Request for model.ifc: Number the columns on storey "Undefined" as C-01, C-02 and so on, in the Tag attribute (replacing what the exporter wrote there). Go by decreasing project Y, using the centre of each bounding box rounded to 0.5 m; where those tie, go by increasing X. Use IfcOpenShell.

First a look at what the model holds.

```python
import ifcopenshell
import ifcopenshell.util.element
import ifcopenshell.util.placement

model = ifcopenshell.open("model.ifc")
print(model.schema)
storey = next(s for s in model.by_type("IfcBuildingStorey") if s.Name == "Undefined")
columns = [e for e in ifcopenshell.util.element.get_decomposition(storey) if e.is_a("IfcColumn")]
for e in sorted(columns, key=lambda e: e.id()):
    origin = ifcopenshell.util.placement.get_local_placement(e.ObjectPlacement)[:3, 3]
    print(e.id(), e.Tag, e.Name, origin.round(2) + 0.0, sep=" | ")
```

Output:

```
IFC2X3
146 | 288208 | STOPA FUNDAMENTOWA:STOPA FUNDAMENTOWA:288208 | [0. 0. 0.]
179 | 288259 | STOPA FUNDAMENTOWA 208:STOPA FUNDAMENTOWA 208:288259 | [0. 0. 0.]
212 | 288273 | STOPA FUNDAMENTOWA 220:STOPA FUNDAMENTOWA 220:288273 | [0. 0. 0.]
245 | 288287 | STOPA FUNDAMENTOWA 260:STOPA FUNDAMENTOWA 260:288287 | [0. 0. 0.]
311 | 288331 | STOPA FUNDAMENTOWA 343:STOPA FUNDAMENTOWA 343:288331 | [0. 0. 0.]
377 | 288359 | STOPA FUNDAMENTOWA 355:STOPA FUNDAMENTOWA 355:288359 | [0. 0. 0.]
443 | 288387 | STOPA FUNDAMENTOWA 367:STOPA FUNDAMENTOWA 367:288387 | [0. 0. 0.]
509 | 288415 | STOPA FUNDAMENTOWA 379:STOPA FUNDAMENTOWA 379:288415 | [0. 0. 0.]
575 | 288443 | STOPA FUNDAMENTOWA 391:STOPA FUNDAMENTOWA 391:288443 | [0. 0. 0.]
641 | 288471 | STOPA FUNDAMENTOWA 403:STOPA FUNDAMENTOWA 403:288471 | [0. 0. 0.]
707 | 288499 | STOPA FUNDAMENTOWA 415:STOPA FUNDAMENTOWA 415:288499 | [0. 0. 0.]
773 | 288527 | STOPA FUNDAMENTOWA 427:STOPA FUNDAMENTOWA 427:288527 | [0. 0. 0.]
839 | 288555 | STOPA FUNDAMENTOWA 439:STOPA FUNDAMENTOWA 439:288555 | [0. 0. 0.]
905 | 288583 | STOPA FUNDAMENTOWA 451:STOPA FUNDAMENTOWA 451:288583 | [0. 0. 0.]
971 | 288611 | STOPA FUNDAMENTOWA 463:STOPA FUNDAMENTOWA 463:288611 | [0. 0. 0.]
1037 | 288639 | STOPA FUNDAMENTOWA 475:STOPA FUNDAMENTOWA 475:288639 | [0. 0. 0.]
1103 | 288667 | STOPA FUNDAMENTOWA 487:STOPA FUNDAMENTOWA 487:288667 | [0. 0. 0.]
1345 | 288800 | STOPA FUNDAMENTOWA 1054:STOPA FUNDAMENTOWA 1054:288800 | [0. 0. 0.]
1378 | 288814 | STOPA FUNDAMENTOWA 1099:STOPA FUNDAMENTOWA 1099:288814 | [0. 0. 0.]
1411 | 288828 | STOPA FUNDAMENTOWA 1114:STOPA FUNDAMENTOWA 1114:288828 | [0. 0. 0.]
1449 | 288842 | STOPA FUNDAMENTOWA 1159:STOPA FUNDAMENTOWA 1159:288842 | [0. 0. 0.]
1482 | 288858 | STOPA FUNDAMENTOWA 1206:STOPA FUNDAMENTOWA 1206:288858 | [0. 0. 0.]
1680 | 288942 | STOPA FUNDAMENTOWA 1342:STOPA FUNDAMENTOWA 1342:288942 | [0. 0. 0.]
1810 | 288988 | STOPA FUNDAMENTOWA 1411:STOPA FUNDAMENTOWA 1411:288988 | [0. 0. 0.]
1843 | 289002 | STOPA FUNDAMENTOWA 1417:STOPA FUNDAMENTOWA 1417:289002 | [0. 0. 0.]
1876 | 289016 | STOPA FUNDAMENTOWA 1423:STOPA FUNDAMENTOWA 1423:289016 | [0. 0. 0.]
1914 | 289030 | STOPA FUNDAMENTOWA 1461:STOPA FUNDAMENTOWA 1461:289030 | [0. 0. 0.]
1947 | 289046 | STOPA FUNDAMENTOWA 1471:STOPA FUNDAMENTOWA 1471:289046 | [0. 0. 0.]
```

```python
import ifcopenshell
import ifcopenshell.geom
import ifcopenshell.util.element
import ifcopenshell.util.shape

model = ifcopenshell.open("model.ifc")
settings = ifcopenshell.geom.settings()
settings.set("use-world-coords", True)


def centre(element):
    shape = ifcopenshell.geom.create_shape(settings, element)
    return ifcopenshell.util.shape.get_bbox_centroid(shape.geometry)


storey = next(s for s in model.by_type("IfcBuildingStorey") if s.Name == "Undefined")
columns = [e for e in ifcopenshell.util.element.get_decomposition(storey) if e.is_a("IfcColumn")]

# Insertion points can sit at a corner or the storey origin, so sort by the geometry (in metres).
centres = {e: centre(e) for e in columns}
columns.sort(key=lambda e: (-round(centres[e][1] / 0.5), centres[e][0]))

for i, e in enumerate(columns, start=1):
    number = f"C-{i:02d}"
    e.Tag = number
    print(e.id(), number)

model.write("model_rev.ifc")
```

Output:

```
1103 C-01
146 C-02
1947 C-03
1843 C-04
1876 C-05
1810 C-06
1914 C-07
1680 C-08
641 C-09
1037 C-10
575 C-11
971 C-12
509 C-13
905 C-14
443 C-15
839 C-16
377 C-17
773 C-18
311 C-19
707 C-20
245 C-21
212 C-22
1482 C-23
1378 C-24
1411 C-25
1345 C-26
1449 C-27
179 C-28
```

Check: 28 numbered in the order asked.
